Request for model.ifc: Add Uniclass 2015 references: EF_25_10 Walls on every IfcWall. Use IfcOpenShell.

First a look at what the model holds.

```python
import ifcopenshell

model = ifcopenshell.open("model.ifc")
print(model.schema)
print("classifications:", [c.Name for c in model.by_type("IfcClassification")])
for ifc_class in ("IfcDoor", "IfcRoof", "IfcStair", "IfcWall", "IfcWindow"):
    print(ifc_class, len(model.by_type(ifc_class)))
```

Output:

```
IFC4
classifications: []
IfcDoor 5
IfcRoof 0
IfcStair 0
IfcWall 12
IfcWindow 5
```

```python
import ifcopenshell
import ifcopenshell.api.classification

model = ifcopenshell.open("model.ifc")

system = ifcopenshell.api.classification.add_classification(model, classification="Uniclass 2015")

codes = {
    "IfcWall": ("EF_25_10", "Walls"),
}
for ifc_class, (code, name) in codes.items():
    products = model.by_type(ifc_class)
    ifcopenshell.api.classification.add_reference(
        model, products=products, classification=system, identification=code, name=name
    )
    print(code, len(products))

model.write("model_rev.ifc")
```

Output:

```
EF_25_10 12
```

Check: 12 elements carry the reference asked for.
